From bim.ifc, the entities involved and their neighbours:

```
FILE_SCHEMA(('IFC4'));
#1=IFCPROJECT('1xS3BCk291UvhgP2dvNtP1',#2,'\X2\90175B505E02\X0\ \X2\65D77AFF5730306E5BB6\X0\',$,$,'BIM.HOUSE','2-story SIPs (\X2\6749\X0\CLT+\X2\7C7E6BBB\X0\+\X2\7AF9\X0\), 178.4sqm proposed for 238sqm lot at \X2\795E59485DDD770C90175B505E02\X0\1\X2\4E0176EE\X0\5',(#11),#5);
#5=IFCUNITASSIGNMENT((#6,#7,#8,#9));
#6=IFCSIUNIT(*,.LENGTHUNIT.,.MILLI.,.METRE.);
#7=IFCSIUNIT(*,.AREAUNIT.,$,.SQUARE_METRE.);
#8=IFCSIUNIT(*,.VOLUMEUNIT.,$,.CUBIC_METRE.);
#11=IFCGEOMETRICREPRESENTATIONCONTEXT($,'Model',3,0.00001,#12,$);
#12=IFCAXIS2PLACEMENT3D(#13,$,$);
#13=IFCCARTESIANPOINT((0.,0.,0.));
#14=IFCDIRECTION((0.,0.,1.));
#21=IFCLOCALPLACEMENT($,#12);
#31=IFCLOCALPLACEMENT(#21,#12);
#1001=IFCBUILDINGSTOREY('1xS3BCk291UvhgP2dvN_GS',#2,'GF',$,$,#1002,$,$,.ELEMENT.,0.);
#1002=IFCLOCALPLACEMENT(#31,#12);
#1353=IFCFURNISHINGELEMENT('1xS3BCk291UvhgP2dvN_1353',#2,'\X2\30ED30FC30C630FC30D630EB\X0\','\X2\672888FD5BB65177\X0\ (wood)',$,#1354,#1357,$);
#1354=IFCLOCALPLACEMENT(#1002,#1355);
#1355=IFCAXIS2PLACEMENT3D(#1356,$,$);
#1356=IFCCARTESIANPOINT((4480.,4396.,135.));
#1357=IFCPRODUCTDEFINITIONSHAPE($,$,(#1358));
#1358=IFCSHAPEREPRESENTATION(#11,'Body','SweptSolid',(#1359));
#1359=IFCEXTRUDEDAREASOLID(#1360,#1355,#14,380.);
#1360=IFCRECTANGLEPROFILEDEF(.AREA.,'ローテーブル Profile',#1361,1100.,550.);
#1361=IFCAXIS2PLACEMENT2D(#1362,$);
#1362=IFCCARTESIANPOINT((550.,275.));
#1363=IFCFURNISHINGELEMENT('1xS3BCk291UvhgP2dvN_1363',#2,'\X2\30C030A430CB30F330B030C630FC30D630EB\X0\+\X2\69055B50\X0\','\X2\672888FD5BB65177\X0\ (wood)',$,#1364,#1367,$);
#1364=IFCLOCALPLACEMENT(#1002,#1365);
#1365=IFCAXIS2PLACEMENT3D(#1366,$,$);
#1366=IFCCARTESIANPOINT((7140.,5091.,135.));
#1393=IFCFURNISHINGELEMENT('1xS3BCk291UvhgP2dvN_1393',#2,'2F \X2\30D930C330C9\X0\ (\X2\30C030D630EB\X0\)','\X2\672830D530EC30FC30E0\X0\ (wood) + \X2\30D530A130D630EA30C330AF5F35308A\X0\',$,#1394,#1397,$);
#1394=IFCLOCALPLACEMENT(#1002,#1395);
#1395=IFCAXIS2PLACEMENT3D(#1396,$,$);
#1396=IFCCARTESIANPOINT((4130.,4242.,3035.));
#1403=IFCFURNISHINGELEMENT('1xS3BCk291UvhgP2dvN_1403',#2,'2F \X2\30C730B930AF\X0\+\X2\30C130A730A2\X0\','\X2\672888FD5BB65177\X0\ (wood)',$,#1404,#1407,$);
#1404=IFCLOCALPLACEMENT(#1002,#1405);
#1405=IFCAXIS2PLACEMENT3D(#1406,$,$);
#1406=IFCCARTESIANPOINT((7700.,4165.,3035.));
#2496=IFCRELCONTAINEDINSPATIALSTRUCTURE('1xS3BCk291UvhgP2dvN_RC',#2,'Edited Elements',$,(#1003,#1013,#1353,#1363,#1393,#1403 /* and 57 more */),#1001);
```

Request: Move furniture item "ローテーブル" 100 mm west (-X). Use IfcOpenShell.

```python
import ifcopenshell
import ifcopenshell.api.geometry
import ifcopenshell.util.placement
import ifcopenshell.util.unit

model = ifcopenshell.open("bim.ifc")
unit_scale = ifcopenshell.util.unit.calculate_unit_scale(model)

item = model.by_id(1353)
matrix = ifcopenshell.util.placement.get_local_placement(item.ObjectPlacement)
matrix[0, 3] -= 0.1 / unit_scale
ifcopenshell.api.geometry.edit_object_placement(model, product=item, matrix=matrix, is_si=False)

print(ifcopenshell.util.placement.get_local_placement(item.ObjectPlacement).round(3) + 0.0)

model.write("bim-out.ifc")
```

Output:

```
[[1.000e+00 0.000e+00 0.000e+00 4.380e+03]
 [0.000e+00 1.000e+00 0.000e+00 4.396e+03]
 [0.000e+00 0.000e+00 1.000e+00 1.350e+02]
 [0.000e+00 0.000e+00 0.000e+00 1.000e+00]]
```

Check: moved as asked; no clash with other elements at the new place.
